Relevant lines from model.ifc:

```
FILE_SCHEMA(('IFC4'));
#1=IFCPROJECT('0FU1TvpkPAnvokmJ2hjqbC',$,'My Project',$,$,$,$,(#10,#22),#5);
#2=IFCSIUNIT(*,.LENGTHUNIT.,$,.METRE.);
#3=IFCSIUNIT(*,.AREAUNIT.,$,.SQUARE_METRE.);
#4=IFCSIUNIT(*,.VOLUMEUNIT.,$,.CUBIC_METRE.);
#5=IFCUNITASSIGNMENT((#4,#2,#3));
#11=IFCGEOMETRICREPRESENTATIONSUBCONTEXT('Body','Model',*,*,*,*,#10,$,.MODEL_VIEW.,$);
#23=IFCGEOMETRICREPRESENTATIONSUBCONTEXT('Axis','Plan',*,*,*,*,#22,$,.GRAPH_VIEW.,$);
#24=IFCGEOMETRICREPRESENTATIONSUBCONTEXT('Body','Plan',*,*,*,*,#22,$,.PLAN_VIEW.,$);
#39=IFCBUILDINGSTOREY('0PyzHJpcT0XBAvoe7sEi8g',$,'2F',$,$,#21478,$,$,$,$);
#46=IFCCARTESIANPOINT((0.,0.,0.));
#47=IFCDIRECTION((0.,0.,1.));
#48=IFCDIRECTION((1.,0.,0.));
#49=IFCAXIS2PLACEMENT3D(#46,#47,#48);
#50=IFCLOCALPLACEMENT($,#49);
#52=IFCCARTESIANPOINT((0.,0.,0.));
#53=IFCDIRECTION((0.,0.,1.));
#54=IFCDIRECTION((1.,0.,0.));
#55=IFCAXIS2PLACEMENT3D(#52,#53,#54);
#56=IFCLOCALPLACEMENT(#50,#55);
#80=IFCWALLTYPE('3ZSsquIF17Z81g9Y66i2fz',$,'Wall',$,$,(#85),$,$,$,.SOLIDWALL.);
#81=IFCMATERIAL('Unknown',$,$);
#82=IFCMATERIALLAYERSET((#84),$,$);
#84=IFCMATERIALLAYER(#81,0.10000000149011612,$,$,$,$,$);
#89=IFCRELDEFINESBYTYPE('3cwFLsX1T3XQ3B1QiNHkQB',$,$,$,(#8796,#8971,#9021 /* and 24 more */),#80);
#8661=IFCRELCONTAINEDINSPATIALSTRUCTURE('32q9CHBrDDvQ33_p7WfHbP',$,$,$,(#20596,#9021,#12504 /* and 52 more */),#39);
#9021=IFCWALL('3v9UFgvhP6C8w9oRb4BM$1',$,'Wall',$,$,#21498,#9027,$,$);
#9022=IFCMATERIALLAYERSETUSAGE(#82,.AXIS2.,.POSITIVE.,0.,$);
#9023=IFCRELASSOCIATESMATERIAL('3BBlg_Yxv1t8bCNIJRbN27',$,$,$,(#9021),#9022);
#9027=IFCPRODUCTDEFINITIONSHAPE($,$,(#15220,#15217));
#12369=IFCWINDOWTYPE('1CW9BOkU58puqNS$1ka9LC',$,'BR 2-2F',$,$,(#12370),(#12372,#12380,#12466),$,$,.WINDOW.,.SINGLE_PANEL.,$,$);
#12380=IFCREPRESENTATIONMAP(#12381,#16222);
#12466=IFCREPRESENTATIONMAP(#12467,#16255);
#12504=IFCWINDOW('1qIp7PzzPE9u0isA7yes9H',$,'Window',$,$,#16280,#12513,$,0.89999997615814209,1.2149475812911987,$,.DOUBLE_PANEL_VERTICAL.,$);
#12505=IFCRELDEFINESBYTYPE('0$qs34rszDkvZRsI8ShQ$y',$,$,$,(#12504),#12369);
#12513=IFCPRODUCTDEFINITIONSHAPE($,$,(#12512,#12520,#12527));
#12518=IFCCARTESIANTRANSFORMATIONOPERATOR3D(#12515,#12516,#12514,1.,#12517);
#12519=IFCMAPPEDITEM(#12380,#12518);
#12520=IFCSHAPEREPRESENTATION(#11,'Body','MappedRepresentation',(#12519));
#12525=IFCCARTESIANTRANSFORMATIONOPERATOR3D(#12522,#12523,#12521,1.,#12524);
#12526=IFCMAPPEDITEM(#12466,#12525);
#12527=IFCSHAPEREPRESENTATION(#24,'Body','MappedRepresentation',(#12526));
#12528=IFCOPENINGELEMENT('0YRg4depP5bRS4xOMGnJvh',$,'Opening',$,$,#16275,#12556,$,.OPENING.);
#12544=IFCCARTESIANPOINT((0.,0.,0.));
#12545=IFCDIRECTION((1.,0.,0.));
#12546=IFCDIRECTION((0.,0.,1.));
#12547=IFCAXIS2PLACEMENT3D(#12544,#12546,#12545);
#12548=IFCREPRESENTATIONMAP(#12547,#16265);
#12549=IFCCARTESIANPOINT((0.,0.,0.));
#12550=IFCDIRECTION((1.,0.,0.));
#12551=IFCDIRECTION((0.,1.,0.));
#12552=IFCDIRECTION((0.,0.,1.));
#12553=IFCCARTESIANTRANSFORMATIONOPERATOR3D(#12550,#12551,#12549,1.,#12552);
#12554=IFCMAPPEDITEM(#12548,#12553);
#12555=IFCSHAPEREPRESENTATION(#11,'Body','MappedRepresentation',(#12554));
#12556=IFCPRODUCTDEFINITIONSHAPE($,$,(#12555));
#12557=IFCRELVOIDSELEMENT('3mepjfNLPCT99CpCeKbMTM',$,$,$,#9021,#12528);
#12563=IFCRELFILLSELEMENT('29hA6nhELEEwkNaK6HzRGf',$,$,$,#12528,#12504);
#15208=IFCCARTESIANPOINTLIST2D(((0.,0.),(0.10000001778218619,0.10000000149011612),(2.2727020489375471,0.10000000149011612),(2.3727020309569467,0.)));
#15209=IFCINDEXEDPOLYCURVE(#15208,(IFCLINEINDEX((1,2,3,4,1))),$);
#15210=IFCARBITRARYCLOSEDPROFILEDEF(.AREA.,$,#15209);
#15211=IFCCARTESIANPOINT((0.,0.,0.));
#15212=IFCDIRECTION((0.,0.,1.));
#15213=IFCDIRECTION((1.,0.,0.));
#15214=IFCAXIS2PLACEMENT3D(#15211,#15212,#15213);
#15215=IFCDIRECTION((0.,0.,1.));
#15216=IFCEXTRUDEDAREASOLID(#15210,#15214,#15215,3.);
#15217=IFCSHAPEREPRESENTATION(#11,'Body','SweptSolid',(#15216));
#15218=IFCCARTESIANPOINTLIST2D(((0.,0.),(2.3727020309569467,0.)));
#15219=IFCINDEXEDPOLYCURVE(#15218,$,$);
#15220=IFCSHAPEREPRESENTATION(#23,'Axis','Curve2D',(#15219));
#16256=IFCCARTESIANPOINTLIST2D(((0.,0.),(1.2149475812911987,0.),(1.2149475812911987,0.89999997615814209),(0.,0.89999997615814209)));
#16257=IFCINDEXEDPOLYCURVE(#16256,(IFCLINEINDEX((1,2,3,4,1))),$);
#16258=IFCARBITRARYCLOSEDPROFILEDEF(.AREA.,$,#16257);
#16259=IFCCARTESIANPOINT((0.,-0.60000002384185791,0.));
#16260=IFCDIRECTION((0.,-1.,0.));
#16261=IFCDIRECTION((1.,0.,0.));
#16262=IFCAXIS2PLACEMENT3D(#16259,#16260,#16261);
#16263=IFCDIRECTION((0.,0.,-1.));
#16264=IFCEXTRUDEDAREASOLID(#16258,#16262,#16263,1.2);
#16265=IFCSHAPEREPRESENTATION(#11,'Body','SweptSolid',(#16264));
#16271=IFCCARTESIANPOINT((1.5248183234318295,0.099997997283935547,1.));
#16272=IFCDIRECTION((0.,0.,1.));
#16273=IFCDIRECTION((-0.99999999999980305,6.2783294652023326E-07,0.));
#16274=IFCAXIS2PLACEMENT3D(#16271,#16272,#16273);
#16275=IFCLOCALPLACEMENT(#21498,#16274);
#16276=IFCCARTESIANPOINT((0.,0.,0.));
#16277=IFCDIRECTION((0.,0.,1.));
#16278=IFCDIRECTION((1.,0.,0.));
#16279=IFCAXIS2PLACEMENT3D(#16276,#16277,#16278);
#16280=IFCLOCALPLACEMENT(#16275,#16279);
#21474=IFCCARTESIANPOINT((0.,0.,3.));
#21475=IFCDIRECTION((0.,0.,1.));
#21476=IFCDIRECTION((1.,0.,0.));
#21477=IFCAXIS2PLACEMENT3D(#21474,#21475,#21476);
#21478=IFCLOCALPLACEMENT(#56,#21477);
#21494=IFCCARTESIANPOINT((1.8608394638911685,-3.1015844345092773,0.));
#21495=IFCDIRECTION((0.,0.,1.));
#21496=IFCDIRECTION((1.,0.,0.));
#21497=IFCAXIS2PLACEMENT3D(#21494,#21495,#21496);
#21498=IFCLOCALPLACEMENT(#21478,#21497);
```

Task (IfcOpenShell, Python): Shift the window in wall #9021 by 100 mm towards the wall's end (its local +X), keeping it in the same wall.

```python
import ifcopenshell
import ifcopenshell.api.geometry
import ifcopenshell.util.placement
import ifcopenshell.util.unit

model = ifcopenshell.open("model.ifc")
unit_scale = ifcopenshell.util.unit.calculate_unit_scale(model)

window = model.by_guid("1qIp7PzzPE9u0isA7yes9H")
opening = window.FillsVoids[0].RelatingOpeningElement
wall = opening.VoidsElements[0].RelatingBuildingElement

wall_matrix = ifcopenshell.util.placement.get_local_placement(wall.ObjectPlacement)
shift = wall_matrix[:3, 0] * 0.1 / unit_scale
before = ifcopenshell.util.placement.get_local_placement(window.ObjectPlacement)[:3, 3].copy()

# The window is placed relative to its opening, so it follows when the opening moves.
matrix = ifcopenshell.util.placement.get_local_placement(opening.ObjectPlacement)
matrix[:3, 3] += shift
ifcopenshell.api.geometry.edit_object_placement(
    model, product=opening, matrix=matrix, is_si=False, should_transform_children=True
)

after = ifcopenshell.util.placement.get_local_placement(window.ObjectPlacement)[:3, 3]
print("window moved by", (after - before).round(3) + 0.0)

model.write("model_v2.ifc")
```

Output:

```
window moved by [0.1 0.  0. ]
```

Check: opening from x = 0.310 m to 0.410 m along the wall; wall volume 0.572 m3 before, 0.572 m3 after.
